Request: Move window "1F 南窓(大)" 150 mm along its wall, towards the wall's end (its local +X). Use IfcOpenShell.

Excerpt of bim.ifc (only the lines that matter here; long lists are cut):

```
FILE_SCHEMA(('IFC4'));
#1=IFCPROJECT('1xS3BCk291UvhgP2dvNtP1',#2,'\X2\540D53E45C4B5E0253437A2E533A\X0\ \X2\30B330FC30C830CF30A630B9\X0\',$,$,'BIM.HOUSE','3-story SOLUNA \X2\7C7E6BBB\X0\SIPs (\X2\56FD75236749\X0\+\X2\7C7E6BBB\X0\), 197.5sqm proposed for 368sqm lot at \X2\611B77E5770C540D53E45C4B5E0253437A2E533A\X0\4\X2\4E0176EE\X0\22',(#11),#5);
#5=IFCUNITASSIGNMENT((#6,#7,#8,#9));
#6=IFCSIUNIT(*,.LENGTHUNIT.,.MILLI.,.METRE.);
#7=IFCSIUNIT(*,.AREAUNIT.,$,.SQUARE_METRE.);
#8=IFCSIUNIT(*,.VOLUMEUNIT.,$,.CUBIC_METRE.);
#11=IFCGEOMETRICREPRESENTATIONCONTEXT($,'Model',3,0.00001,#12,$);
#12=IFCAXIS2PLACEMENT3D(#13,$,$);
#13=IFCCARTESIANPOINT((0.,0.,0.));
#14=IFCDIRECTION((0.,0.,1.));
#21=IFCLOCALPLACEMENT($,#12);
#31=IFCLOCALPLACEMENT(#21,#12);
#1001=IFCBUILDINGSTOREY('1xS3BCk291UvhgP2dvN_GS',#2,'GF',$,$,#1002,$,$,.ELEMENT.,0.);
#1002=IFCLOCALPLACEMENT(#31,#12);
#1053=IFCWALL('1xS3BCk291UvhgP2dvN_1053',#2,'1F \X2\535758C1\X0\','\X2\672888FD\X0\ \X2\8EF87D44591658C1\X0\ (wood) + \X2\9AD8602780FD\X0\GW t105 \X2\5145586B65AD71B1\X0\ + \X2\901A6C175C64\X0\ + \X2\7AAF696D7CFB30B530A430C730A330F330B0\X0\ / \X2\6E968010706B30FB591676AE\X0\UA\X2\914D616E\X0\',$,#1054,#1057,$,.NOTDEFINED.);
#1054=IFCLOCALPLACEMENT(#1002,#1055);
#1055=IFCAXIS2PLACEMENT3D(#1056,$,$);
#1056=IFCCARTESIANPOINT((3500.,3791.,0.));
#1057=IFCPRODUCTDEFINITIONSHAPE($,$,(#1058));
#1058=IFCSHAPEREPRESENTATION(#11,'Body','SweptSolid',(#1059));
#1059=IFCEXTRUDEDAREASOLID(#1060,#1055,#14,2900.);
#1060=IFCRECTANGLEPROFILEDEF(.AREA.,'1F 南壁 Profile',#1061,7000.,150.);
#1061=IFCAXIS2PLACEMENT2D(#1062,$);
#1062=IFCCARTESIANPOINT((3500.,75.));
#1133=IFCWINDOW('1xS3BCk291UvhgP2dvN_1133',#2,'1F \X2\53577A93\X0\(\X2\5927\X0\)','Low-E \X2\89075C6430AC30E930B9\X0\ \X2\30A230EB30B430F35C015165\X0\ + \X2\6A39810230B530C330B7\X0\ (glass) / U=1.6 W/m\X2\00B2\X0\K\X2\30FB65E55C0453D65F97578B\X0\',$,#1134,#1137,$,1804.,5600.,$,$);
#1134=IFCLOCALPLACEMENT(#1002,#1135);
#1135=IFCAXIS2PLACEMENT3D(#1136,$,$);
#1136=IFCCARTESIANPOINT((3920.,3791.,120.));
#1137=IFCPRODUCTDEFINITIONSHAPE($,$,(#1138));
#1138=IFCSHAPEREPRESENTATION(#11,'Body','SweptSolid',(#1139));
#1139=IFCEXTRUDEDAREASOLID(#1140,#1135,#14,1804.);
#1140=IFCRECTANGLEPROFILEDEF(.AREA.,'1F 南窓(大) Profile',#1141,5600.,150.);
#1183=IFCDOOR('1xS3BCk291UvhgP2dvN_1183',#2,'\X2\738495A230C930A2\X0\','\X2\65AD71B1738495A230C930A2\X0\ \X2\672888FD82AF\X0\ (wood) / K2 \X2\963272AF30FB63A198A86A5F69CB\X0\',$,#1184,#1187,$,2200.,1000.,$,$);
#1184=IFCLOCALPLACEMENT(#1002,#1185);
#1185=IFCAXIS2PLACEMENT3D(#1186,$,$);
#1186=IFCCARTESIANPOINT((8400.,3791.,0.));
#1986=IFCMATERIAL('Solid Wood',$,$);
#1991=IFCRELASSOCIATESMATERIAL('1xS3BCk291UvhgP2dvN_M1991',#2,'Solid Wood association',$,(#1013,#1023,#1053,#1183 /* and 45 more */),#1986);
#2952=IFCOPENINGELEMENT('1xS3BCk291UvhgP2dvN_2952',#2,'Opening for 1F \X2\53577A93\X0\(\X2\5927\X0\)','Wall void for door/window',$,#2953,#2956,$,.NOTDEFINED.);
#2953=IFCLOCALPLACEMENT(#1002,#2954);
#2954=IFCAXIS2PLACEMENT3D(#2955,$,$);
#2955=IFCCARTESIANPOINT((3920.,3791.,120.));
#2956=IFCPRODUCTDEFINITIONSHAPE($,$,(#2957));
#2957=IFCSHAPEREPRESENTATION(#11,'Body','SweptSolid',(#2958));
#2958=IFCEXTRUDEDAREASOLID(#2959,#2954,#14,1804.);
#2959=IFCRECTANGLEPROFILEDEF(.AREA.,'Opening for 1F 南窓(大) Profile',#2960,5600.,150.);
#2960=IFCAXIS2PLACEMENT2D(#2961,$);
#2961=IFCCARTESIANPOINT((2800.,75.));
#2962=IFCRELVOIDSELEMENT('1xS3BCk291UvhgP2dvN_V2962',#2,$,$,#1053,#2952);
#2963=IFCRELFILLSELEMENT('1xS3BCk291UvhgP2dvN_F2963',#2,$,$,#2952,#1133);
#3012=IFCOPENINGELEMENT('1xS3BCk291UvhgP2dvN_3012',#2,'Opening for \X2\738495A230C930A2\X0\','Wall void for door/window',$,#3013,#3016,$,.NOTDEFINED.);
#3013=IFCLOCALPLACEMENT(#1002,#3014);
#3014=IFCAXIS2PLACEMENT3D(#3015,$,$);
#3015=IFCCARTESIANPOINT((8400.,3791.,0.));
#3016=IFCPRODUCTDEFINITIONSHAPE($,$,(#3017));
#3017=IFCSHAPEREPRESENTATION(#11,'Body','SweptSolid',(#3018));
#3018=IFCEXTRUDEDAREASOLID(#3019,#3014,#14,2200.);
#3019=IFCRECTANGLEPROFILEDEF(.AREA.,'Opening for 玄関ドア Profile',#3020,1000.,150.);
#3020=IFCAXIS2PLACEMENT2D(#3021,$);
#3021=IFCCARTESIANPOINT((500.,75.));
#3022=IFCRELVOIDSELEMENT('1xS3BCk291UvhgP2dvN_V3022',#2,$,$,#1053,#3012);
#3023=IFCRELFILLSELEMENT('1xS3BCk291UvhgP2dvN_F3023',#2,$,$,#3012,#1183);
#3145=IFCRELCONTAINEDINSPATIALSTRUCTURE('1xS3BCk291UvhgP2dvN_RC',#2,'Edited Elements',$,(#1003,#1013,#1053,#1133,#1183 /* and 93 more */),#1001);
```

```python
import ifcopenshell
import ifcopenshell.api.geometry
import ifcopenshell.util.placement
import ifcopenshell.util.unit

model = ifcopenshell.open("bim.ifc")
unit_scale = ifcopenshell.util.unit.calculate_unit_scale(model)

window = model.by_guid("1xS3BCk291UvhgP2dvN_1133")
opening = window.FillsVoids[0].RelatingOpeningElement
wall = opening.VoidsElements[0].RelatingBuildingElement

wall_matrix = ifcopenshell.util.placement.get_local_placement(wall.ObjectPlacement)
shift = wall_matrix[:3, 0] * 0.15 / unit_scale
before = ifcopenshell.util.placement.get_local_placement(window.ObjectPlacement)[:3, 3].copy()

# The window is not placed relative to its opening, so move both.
for product in (opening, window):
    matrix = ifcopenshell.util.placement.get_local_placement(product.ObjectPlacement)
    matrix[:3, 3] += shift
    ifcopenshell.api.geometry.edit_object_placement(model, product=product, matrix=matrix, is_si=False)

after = ifcopenshell.util.placement.get_local_placement(window.ObjectPlacement)[:3, 3]
print("window moved by", (after - before).round(3) + 0.0)

model.write("bim_edited.ifc")
```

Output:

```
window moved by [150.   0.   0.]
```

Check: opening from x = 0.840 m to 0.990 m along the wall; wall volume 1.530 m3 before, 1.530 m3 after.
